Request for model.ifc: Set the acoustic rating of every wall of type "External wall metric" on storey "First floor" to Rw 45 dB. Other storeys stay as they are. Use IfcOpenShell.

First a look at what the model holds.

```python
import ifcopenshell
import ifcopenshell.util.element

model = ifcopenshell.open("model.ifc")
print(model.schema)
storey = next(s for s in model.by_type("IfcBuildingStorey") if s.Name == "First floor")
walls = [e for e in ifcopenshell.util.element.get_decomposition(storey) if e.is_a("IfcWall")]
seen = {}
for e in walls:
    element_type = ifcopenshell.util.element.get_type(e)
    key = (element_type.Name if element_type != e and element_type else None, ifcopenshell.util.element.get_pset(e, "Pset_WallCommon", "AcousticRating"))
    seen[key] = seen.get(key, 0) + 1
for (name, value), count in sorted(seen.items(), key=str):
    print(count, "x", name, "|", value)
```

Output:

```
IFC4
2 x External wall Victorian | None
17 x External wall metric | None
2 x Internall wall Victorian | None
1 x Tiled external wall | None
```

```python
import ifcopenshell
import ifcopenshell.api.pset
import ifcopenshell.util.element

model = ifcopenshell.open("model.ifc")

storey = next(s for s in model.by_type("IfcBuildingStorey") if s.Name == "First floor")
walls = [e for e in ifcopenshell.util.element.get_decomposition(storey) if e.is_a("IfcWall")]

count = 0
for e in walls:
    element_type = ifcopenshell.util.element.get_type(e)
    if element_type in (None, e) or element_type.Name != "External wall metric":
        continue
    # add_pset returns the element's existing set when there is one.
    pset = ifcopenshell.api.pset.add_pset(model, product=e, name="Pset_WallCommon")
    ifcopenshell.api.pset.edit_pset(model, pset=pset, properties={"AcousticRating": "Rw 45 dB"})
    count += 1

print(count, "walls updated")

model.write("model_edited.ifc")
```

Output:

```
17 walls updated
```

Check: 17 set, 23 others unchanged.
